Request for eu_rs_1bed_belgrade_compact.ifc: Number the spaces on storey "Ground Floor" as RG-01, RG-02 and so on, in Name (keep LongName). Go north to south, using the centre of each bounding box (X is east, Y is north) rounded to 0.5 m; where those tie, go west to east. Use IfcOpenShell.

First a look at what the model holds.

```python
import ifcopenshell
import ifcopenshell.util.element
import ifcopenshell.util.placement

model = ifcopenshell.open("eu_rs_1bed_belgrade_compact.ifc")
print(model.schema)
storey = next(s for s in model.by_type("IfcBuildingStorey") if s.Name == "Ground Floor")
spaces = [e for e in ifcopenshell.util.element.get_decomposition(storey) if e.is_a("IfcSpace")]
for e in sorted(spaces, key=lambda e: e.id()):
    origin = ifcopenshell.util.placement.get_local_placement(e.ObjectPlacement)[:3, 3]
    print(e.id(), e.Name, e.LongName, origin.round(2) + 0.0, sep=" | ")
```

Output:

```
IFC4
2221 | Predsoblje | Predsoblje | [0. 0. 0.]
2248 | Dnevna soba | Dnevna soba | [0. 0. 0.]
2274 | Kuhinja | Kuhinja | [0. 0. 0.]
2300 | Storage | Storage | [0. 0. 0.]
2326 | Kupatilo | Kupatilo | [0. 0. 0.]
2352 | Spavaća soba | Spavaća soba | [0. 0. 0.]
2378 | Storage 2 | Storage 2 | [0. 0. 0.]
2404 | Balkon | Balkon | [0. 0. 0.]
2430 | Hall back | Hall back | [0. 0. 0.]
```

```python
import ifcopenshell
import ifcopenshell.geom
import ifcopenshell.util.element
import ifcopenshell.util.shape

model = ifcopenshell.open("eu_rs_1bed_belgrade_compact.ifc")
settings = ifcopenshell.geom.settings()
settings.set("use-world-coords", True)


def centre(element):
    shape = ifcopenshell.geom.create_shape(settings, element)
    return ifcopenshell.util.shape.get_bbox_centroid(shape.geometry)


storey = next(s for s in model.by_type("IfcBuildingStorey") if s.Name == "Ground Floor")
spaces = [e for e in ifcopenshell.util.element.get_decomposition(storey) if e.is_a("IfcSpace")]

# Insertion points can sit at a corner or the storey origin, so sort by the geometry (in metres).
centres = {e: centre(e) for e in spaces}
spaces.sort(key=lambda e: (-round(centres[e][1] / 0.5), centres[e][0]))

for i, e in enumerate(spaces, start=1):
    number = f"RG-{i:02d}"
    e.Name = number
    print(e.id(), number)

model.write("eu_rs_1bed_belgrade_compact-out.ifc")
```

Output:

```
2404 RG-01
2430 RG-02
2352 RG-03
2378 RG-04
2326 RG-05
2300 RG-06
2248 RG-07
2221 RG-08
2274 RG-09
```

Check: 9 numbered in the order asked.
